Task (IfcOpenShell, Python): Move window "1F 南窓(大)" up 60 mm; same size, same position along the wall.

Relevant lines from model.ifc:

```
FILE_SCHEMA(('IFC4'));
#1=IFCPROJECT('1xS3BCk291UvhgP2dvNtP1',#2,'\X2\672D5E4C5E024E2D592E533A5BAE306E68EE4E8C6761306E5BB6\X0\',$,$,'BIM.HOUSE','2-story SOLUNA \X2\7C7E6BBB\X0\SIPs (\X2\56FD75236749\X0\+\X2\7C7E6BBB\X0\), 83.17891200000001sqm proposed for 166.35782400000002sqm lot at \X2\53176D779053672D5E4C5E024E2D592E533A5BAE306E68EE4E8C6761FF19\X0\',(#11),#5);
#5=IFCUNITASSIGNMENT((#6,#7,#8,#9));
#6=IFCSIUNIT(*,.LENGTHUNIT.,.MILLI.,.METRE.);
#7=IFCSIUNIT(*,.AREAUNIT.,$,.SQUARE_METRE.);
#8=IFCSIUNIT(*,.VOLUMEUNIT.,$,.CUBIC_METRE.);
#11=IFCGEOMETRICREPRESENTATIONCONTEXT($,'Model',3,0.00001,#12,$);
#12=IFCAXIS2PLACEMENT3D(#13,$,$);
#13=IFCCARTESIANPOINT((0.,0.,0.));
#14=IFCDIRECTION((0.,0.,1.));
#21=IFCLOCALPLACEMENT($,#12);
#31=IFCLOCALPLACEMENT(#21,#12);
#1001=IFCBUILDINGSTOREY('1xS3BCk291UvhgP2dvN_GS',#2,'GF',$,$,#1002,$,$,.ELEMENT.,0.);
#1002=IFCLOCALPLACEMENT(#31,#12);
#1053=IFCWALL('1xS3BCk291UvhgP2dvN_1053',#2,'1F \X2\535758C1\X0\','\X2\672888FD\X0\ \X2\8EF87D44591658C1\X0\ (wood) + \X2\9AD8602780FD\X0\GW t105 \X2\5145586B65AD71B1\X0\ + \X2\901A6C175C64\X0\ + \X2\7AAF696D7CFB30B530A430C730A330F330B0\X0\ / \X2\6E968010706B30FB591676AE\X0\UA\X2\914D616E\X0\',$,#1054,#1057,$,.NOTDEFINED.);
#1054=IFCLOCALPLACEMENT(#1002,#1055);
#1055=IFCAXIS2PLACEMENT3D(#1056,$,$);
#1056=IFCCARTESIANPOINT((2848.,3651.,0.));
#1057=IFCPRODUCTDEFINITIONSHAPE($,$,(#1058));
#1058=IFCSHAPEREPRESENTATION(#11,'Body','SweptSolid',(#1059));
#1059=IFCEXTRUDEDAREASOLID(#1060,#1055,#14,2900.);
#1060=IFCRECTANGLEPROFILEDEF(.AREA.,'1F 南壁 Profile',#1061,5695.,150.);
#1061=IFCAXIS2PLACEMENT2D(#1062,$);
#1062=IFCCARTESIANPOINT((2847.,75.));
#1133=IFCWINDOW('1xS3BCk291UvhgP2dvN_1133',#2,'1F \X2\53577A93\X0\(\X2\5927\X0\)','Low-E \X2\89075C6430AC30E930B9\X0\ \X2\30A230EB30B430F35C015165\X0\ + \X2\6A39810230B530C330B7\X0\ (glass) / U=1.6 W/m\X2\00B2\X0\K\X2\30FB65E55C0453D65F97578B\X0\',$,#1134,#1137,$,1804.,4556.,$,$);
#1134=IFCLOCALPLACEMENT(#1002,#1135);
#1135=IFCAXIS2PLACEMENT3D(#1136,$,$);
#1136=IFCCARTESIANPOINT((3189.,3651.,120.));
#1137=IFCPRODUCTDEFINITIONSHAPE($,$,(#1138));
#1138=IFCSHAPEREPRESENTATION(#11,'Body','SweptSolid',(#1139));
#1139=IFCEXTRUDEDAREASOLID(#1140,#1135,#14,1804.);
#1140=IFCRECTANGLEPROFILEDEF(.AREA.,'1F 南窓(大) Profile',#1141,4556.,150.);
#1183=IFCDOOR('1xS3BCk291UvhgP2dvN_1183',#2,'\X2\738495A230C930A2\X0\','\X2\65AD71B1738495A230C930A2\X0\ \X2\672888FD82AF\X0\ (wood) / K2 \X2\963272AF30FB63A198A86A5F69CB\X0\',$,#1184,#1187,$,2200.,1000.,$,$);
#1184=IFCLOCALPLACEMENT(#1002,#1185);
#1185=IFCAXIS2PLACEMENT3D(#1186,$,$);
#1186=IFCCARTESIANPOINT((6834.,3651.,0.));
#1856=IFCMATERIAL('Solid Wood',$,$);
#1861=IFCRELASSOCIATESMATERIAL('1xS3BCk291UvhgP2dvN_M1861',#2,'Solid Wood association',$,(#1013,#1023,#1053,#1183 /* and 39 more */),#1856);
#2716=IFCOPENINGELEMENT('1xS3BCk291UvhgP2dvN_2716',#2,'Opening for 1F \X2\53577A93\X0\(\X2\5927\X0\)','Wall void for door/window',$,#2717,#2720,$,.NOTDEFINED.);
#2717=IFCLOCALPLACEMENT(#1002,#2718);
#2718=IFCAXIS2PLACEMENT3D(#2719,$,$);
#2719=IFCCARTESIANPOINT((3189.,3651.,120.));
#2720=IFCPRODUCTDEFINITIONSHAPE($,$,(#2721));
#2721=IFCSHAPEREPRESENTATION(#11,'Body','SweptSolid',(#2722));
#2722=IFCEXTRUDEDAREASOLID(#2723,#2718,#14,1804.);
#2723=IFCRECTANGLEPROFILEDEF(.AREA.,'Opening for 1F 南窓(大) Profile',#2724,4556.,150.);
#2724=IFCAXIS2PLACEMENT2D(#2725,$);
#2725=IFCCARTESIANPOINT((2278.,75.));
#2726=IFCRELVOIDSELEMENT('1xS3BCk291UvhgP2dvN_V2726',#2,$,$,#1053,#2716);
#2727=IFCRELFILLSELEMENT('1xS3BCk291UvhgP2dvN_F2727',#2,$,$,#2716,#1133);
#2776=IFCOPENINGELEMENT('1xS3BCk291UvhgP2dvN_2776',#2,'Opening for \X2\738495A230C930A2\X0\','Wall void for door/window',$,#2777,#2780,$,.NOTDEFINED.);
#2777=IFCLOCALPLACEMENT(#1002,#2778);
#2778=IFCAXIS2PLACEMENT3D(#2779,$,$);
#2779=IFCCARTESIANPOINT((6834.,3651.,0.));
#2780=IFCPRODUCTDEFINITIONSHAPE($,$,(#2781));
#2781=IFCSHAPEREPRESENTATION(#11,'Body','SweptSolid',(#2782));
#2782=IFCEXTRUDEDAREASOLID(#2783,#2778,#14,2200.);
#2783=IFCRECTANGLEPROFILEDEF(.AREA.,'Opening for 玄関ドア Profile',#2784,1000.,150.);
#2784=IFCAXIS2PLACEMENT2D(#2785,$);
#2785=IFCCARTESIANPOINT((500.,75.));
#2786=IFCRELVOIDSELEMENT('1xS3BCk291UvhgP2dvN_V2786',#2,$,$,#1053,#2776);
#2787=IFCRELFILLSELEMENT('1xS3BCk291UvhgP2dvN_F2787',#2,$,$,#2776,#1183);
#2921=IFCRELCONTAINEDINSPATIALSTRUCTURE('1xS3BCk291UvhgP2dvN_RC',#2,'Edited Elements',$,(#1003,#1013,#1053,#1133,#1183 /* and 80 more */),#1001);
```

```python
import numpy as np
import ifcopenshell
import ifcopenshell.api.geometry
import ifcopenshell.util.placement
import ifcopenshell.util.unit

model = ifcopenshell.open("model.ifc")
unit_scale = ifcopenshell.util.unit.calculate_unit_scale(model)

window = model.by_guid("1xS3BCk291UvhgP2dvN_1133")
opening = window.FillsVoids[0].RelatingOpeningElement
dz = 0.06 / unit_scale

shift = np.array([0.0, 0.0, dz])
# The window is not placed relative to its opening, so move both.
for product in (opening, window):
    matrix = ifcopenshell.util.placement.get_local_placement(product.ObjectPlacement)
    matrix[:3, 3] += shift
    ifcopenshell.api.geometry.edit_object_placement(model, product=product, matrix=matrix, is_si=False)

print(f"moved by {dz * unit_scale:+.3f} m")

model.write("model-out.ifc")
```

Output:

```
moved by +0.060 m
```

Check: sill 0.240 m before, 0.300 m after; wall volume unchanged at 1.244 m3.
